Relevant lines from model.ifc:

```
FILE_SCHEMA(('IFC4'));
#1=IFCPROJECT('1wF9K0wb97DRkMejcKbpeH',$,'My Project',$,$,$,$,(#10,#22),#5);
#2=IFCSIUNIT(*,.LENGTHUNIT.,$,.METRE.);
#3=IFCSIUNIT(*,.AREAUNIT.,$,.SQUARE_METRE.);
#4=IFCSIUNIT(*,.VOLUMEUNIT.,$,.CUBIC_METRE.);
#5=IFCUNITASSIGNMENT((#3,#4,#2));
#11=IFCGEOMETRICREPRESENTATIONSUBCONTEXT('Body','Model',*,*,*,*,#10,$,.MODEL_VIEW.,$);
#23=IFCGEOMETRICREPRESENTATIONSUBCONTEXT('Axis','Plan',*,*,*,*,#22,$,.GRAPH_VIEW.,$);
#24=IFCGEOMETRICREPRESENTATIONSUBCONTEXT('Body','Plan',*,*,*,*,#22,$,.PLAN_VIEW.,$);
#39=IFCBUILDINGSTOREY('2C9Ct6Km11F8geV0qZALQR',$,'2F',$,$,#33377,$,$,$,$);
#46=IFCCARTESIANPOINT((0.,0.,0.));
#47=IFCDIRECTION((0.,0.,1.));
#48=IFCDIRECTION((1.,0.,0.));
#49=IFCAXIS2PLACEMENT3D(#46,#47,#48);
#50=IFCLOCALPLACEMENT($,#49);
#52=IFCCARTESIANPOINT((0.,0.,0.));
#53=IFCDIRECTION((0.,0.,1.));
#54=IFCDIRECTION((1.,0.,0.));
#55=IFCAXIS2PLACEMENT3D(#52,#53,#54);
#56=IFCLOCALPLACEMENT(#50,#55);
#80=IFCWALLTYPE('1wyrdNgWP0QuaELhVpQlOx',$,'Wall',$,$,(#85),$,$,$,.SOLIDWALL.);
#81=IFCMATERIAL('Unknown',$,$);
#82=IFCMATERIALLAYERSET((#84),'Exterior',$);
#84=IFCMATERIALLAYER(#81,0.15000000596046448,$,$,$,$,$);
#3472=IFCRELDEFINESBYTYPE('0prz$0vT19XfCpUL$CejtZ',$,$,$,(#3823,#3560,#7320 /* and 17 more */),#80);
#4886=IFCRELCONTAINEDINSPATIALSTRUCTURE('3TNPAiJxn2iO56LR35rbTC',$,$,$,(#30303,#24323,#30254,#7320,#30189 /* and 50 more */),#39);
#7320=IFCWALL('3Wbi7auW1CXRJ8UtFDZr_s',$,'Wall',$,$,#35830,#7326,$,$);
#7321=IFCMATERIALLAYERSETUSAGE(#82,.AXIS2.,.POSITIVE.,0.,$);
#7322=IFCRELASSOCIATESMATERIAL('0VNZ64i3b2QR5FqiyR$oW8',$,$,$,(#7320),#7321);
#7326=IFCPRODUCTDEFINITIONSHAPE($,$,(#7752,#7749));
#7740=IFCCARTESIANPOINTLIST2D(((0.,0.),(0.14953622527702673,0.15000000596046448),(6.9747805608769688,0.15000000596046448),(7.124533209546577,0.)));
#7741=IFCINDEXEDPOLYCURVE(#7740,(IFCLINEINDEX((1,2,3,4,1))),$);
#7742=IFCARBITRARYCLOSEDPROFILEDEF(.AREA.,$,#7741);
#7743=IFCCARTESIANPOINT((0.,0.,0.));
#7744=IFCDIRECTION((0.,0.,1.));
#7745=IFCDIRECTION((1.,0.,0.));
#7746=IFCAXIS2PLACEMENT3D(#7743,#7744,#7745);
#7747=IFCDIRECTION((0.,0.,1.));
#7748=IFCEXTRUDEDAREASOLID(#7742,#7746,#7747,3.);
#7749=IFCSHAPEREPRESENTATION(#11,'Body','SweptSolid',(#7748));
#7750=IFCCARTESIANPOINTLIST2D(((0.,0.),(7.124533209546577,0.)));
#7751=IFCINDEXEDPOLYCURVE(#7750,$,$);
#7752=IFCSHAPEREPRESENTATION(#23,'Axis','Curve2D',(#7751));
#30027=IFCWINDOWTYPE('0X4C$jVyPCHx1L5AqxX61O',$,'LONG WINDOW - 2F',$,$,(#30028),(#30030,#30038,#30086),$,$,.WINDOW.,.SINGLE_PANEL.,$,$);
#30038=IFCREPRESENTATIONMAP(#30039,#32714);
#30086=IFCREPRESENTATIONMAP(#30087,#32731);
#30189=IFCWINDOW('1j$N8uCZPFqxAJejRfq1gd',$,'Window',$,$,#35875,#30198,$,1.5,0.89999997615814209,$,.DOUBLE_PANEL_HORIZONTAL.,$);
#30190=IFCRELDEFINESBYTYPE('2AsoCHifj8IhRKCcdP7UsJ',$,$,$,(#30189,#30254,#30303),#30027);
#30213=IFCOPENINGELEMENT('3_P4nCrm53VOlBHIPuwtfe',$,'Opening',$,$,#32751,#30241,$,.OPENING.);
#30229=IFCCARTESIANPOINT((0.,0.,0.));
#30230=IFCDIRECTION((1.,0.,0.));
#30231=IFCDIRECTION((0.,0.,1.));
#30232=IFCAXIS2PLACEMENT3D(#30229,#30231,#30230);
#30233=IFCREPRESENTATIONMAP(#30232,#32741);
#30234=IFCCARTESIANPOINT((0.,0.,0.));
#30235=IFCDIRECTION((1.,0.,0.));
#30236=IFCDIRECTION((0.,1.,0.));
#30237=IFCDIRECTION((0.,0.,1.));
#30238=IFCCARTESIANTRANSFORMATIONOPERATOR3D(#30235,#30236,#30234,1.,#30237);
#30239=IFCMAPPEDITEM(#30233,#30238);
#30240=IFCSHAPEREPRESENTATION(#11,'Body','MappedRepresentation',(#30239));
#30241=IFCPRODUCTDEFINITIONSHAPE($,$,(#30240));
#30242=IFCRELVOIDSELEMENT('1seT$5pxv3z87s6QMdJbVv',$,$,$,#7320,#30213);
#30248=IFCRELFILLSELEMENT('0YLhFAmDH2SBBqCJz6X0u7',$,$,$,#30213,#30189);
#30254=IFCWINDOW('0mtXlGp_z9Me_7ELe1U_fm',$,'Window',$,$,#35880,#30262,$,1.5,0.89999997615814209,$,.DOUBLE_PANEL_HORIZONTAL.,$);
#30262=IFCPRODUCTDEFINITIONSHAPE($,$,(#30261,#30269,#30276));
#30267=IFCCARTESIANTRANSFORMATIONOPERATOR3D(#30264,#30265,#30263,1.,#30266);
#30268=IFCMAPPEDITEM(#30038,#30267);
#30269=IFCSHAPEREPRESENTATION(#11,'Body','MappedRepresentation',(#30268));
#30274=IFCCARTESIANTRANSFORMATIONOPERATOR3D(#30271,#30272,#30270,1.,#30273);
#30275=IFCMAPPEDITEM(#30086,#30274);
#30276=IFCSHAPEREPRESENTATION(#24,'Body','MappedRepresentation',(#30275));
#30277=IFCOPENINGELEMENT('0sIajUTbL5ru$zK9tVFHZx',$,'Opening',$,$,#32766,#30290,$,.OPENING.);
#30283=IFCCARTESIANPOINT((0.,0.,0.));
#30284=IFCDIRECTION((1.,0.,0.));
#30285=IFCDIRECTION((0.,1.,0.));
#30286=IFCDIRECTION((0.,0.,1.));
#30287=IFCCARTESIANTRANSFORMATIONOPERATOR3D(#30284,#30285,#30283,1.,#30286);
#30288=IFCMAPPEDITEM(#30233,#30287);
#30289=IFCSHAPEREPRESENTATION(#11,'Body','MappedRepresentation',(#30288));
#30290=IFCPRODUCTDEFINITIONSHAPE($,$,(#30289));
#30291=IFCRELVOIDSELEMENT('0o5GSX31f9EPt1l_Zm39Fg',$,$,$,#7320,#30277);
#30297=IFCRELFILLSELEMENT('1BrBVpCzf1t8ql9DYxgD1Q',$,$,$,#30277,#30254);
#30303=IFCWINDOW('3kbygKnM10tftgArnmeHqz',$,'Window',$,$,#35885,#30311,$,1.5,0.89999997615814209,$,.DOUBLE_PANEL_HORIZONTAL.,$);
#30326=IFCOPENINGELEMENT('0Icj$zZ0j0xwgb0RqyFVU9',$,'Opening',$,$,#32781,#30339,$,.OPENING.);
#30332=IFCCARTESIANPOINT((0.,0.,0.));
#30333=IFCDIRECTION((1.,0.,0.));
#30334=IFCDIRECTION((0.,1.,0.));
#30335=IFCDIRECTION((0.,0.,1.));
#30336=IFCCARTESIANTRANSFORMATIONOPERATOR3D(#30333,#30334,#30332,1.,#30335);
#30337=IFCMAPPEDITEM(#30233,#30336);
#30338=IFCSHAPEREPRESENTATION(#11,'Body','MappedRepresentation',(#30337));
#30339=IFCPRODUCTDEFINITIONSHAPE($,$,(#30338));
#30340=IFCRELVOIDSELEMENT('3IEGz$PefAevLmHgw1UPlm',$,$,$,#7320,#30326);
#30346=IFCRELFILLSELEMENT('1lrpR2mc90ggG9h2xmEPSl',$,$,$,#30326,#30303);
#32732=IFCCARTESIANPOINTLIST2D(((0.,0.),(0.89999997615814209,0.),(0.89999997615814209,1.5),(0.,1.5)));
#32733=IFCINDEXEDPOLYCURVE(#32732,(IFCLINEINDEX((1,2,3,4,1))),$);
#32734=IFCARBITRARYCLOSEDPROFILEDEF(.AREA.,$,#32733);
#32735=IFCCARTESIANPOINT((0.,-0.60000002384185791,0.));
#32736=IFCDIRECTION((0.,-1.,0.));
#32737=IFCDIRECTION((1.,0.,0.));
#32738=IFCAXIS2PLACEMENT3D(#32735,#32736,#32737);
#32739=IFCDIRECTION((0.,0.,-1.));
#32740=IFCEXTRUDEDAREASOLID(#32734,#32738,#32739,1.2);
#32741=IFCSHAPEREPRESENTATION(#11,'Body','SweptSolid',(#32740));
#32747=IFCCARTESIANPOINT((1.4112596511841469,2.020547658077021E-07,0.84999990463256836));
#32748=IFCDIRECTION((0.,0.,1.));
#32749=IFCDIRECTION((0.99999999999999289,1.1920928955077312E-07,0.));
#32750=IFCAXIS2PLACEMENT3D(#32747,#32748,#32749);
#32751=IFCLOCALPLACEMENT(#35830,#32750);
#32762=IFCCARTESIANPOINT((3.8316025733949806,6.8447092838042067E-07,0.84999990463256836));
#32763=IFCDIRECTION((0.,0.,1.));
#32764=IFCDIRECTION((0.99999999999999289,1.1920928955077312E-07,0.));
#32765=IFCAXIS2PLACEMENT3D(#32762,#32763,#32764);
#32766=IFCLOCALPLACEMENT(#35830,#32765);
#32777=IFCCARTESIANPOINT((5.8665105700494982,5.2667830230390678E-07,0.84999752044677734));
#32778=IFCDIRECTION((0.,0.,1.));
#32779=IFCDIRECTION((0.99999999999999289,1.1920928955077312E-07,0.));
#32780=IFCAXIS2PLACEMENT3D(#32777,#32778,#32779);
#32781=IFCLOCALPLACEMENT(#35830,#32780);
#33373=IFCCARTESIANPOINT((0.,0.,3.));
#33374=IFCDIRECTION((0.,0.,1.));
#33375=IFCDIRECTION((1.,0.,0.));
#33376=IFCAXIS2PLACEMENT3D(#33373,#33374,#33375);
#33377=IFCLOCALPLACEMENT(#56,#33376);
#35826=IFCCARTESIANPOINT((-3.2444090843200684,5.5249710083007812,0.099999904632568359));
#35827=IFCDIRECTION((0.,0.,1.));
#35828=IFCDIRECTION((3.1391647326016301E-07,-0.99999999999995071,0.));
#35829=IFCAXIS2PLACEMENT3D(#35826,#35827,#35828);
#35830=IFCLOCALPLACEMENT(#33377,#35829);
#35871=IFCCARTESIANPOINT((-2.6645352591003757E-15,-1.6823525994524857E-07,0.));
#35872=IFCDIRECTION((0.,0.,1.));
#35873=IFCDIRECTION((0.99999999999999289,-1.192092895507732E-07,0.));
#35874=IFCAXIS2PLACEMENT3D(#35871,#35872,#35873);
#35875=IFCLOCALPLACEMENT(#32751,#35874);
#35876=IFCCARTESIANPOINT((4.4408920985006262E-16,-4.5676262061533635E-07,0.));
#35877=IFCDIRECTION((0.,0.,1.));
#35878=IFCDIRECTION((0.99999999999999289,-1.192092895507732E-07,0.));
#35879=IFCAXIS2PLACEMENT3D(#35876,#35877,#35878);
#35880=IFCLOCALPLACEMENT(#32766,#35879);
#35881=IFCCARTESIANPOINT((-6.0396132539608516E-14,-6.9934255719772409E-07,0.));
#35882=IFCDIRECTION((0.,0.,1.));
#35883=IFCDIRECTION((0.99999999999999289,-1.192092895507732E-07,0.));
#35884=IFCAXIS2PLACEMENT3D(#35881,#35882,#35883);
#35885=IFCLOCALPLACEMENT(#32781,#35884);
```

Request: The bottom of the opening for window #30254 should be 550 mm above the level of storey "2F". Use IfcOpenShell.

```python
import numpy as np
import ifcopenshell
import ifcopenshell.api.geometry
import ifcopenshell.geom
import ifcopenshell.util.element
import ifcopenshell.util.placement
import ifcopenshell.util.shape
import ifcopenshell.util.unit

model = ifcopenshell.open("model.ifc")
unit_scale = ifcopenshell.util.unit.calculate_unit_scale(model)

window = model.by_id(30254)
opening = window.FillsVoids[0].RelatingOpeningElement
storey = ifcopenshell.util.element.get_container(window, ifc_class="IfcBuildingStorey")
level = ifcopenshell.util.placement.get_local_placement(storey.ObjectPlacement)[2, 3]

# The opening's origin need not be at the sill, so measure its lowest point.
shape = ifcopenshell.geom.create_shape(ifcopenshell.geom.settings(), opening)
bottom = ifcopenshell.util.shape.get_shape_bottom_elevation(shape, shape.geometry) / unit_scale
dz = level + 0.55 / unit_scale - bottom

shift = np.array([0.0, 0.0, dz])
# The window is placed relative to its opening, so it follows when the opening moves.
matrix = ifcopenshell.util.placement.get_local_placement(opening.ObjectPlacement)
matrix[:3, 3] += shift
ifcopenshell.api.geometry.edit_object_placement(
    model, product=opening, matrix=matrix, is_si=False, should_transform_children=True
)

print(f"moved by {dz * unit_scale:+.3f} m")

model.write("model_edited.ifc")
```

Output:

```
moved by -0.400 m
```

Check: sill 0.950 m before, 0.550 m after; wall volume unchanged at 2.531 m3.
